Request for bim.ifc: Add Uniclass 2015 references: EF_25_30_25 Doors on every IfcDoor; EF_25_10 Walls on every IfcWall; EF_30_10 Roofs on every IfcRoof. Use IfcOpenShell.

First a look at what the model holds.

```python
import ifcopenshell

model = ifcopenshell.open("bim.ifc")
print(model.schema)
print("classifications:", [c.Name for c in model.by_type("IfcClassification")])
for ifc_class in ("IfcDoor", "IfcRoof", "IfcStair", "IfcWall", "IfcWindow"):
    print(ifc_class, len(model.by_type(ifc_class)))
```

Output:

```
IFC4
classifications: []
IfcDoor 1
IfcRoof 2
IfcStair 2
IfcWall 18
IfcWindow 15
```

```python
import ifcopenshell
import ifcopenshell.api.classification

model = ifcopenshell.open("bim.ifc")

system = ifcopenshell.api.classification.add_classification(model, classification="Uniclass 2015")

codes = {
    "IfcDoor": ("EF_25_30_25", "Doors"),
    "IfcWall": ("EF_25_10", "Walls"),
    "IfcRoof": ("EF_30_10", "Roofs"),
}
for ifc_class, (code, name) in codes.items():
    products = model.by_type(ifc_class)
    ifcopenshell.api.classification.add_reference(
        model, products=products, classification=system, identification=code, name=name
    )
    print(code, len(products))

model.write("bim_rev.ifc")
```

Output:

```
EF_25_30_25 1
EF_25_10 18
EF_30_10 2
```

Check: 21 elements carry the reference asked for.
